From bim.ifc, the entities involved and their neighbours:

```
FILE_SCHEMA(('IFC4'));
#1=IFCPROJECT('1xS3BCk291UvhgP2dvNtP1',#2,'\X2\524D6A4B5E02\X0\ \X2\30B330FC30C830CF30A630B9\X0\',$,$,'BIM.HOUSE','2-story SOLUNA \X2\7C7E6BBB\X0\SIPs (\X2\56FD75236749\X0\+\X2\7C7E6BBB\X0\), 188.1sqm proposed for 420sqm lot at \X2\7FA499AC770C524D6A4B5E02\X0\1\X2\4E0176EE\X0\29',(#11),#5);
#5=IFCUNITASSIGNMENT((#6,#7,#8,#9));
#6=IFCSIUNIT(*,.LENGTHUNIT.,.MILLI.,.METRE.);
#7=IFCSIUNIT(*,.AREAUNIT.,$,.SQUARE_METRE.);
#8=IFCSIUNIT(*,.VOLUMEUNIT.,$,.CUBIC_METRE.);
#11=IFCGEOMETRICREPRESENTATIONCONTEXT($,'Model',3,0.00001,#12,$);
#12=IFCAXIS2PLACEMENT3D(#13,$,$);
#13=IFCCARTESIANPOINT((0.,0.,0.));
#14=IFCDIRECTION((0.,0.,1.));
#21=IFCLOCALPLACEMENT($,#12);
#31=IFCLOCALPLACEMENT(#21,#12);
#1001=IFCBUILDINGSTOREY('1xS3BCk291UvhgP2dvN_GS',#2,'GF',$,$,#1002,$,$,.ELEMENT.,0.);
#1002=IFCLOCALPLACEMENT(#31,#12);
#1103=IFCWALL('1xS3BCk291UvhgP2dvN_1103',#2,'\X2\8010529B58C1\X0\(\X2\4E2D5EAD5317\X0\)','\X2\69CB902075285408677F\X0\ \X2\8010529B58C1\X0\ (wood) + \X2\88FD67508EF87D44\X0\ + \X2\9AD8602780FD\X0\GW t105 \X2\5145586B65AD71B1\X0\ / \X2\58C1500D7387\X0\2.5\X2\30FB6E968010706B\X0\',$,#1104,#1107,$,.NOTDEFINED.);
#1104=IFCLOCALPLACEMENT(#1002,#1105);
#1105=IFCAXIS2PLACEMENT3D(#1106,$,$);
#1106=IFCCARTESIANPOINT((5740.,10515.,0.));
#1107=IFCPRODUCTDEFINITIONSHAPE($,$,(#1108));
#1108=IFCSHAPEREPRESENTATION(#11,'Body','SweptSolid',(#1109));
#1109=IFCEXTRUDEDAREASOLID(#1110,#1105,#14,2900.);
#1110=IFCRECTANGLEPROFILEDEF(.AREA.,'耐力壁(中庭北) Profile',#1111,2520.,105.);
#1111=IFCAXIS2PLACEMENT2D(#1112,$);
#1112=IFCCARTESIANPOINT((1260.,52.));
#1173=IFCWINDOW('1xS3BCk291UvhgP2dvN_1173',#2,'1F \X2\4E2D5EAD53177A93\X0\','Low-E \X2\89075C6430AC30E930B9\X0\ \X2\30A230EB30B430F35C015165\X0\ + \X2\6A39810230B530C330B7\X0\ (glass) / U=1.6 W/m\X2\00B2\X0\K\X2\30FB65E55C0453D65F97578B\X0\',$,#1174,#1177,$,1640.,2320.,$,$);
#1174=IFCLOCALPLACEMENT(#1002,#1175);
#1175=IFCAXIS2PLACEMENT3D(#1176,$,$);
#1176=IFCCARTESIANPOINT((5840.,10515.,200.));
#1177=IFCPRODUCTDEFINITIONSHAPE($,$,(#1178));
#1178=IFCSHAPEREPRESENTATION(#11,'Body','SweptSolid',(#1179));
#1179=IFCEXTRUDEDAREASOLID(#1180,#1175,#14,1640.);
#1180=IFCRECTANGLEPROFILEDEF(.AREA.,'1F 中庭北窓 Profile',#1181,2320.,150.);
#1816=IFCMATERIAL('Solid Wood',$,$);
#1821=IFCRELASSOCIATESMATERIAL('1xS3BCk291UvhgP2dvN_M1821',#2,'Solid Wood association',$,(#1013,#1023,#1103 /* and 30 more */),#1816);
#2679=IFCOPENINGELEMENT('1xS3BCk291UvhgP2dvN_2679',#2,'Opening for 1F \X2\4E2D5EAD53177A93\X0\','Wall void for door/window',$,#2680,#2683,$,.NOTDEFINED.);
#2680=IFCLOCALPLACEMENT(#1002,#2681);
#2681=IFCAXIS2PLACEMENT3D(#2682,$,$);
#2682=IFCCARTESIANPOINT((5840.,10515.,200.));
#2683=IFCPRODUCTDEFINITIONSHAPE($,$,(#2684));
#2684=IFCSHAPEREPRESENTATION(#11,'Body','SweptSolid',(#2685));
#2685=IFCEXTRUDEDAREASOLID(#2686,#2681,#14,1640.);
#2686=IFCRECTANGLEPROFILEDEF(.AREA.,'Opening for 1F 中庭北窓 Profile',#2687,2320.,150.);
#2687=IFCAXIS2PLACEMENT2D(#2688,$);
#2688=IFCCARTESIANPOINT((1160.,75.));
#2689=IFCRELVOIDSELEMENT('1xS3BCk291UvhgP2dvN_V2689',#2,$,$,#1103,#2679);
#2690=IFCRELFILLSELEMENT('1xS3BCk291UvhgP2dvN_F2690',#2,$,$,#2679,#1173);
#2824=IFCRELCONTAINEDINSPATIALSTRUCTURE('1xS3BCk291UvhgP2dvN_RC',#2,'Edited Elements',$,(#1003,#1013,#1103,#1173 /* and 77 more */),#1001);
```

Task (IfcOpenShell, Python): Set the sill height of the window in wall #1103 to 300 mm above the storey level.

```python
import numpy as np
import ifcopenshell
import ifcopenshell.api.geometry
import ifcopenshell.geom
import ifcopenshell.util.element
import ifcopenshell.util.placement
import ifcopenshell.util.shape
import ifcopenshell.util.unit

model = ifcopenshell.open("bim.ifc")
unit_scale = ifcopenshell.util.unit.calculate_unit_scale(model)

window = model.by_guid("1xS3BCk291UvhgP2dvN_1173")
opening = window.FillsVoids[0].RelatingOpeningElement
storey = ifcopenshell.util.element.get_container(window, ifc_class="IfcBuildingStorey")
level = ifcopenshell.util.placement.get_local_placement(storey.ObjectPlacement)[2, 3]

# The opening's origin need not be at the sill, so measure its lowest point.
shape = ifcopenshell.geom.create_shape(ifcopenshell.geom.settings(), opening)
bottom = ifcopenshell.util.shape.get_shape_bottom_elevation(shape, shape.geometry) / unit_scale
dz = level + 0.3 / unit_scale - bottom

shift = np.array([0.0, 0.0, dz])
# The window is not placed relative to its opening, so move both.
for product in (opening, window):
    matrix = ifcopenshell.util.placement.get_local_placement(product.ObjectPlacement)
    matrix[:3, 3] += shift
    ifcopenshell.api.geometry.edit_object_placement(model, product=product, matrix=matrix, is_si=False)

print(f"moved by {dz * unit_scale:+.3f} m")

model.write("bim-out.ifc")
```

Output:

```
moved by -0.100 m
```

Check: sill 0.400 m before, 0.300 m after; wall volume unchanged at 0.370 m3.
